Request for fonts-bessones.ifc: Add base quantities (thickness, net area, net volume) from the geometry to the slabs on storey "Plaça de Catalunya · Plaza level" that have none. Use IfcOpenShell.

First a look at what the model holds.

```python
import ifcopenshell
import ifcopenshell.util.element
import ifcopenshell.util.unit

model = ifcopenshell.open("fonts-bessones.ifc")
print(model.schema)
for unit_type in ("LENGTHUNIT", "AREAUNIT", "VOLUMEUNIT"):
    print(unit_type, ifcopenshell.util.unit.calculate_unit_scale(model, unit_type))
storey = next(s for s in model.by_type("IfcBuildingStorey") if s.Name == "Plaça de Catalunya · Plaza level")
slabs = [e for e in ifcopenshell.util.element.get_decomposition(storey) if e.is_a("IfcSlab")]
for e in sorted(slabs, key=lambda e: e.id()):
    print(e.id(), e.is_a(), e.Name, list(ifcopenshell.util.element.get_psets(e, qtos_only=True)), sep=" | ")
```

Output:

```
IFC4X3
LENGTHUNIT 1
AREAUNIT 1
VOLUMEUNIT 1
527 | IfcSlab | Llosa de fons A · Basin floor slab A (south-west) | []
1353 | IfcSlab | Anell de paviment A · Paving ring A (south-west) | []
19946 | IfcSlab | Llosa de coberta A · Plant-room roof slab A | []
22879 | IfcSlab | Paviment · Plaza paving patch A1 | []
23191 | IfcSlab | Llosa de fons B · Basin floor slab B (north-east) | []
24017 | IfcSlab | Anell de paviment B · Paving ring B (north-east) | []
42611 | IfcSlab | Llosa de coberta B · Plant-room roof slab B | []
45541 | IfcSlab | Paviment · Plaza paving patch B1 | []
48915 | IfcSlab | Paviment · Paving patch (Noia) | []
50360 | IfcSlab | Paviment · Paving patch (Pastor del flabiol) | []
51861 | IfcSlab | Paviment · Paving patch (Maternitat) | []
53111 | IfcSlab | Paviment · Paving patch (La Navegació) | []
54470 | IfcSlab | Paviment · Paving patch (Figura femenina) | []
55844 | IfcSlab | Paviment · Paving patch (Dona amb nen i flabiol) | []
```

```python
import ifcopenshell
import ifcopenshell.api.pset
import ifcopenshell.geom
import ifcopenshell.util.element
import ifcopenshell.util.shape
import ifcopenshell.util.unit

model = ifcopenshell.open("fonts-bessones.ifc")
unit_scale = ifcopenshell.util.unit.calculate_unit_scale(model)
area_scale = ifcopenshell.util.unit.calculate_unit_scale(model, "AREAUNIT")
volume_scale = ifcopenshell.util.unit.calculate_unit_scale(model, "VOLUMEUNIT")
settings = ifcopenshell.geom.settings()

storey = next(s for s in model.by_type("IfcBuildingStorey") if s.Name == "Plaça de Catalunya · Plaza level")
slabs = [e for e in ifcopenshell.util.element.get_decomposition(storey) if e.is_a("IfcSlab")]

for e in sorted(slabs, key=lambda e: e.id()):
    if ifcopenshell.util.element.get_psets(e, qtos_only=True, should_inherit=False):
        continue
    # Geometry comes back in metres, in the element's own axes.
    shape = ifcopenshell.geom.create_shape(settings, e)
    values = {
        "Width": ifcopenshell.util.shape.get_z(shape.geometry) / unit_scale,
        "NetArea": ifcopenshell.util.shape.get_footprint_area(shape.geometry) / area_scale,
        "NetVolume": ifcopenshell.util.shape.get_volume(shape.geometry) / volume_scale,
    }
    qto = ifcopenshell.api.pset.add_qto(model, product=e, name="Qto_SlabBaseQuantities")
    ifcopenshell.api.pset.edit_qto(model, qto=qto, properties=values)
    print(e.id(), {k: round(v, 3) for k, v in values.items()})

model.write("fonts-bessones_v2.ifc")
```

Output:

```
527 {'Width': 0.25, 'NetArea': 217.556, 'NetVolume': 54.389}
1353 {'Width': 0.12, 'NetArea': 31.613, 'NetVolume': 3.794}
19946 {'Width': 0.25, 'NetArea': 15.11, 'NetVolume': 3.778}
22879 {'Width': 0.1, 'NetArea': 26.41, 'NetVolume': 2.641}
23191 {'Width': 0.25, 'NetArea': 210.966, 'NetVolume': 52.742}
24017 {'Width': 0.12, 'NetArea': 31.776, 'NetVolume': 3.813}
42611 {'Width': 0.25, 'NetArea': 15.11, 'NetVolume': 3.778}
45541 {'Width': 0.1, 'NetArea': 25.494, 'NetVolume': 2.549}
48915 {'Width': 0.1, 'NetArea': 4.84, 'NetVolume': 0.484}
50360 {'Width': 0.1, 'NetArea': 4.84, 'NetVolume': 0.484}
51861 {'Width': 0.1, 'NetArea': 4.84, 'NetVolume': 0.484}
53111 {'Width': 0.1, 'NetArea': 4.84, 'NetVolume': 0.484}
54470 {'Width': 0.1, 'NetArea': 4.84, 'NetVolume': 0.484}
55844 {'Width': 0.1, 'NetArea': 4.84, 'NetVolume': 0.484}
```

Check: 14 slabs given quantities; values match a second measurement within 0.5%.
